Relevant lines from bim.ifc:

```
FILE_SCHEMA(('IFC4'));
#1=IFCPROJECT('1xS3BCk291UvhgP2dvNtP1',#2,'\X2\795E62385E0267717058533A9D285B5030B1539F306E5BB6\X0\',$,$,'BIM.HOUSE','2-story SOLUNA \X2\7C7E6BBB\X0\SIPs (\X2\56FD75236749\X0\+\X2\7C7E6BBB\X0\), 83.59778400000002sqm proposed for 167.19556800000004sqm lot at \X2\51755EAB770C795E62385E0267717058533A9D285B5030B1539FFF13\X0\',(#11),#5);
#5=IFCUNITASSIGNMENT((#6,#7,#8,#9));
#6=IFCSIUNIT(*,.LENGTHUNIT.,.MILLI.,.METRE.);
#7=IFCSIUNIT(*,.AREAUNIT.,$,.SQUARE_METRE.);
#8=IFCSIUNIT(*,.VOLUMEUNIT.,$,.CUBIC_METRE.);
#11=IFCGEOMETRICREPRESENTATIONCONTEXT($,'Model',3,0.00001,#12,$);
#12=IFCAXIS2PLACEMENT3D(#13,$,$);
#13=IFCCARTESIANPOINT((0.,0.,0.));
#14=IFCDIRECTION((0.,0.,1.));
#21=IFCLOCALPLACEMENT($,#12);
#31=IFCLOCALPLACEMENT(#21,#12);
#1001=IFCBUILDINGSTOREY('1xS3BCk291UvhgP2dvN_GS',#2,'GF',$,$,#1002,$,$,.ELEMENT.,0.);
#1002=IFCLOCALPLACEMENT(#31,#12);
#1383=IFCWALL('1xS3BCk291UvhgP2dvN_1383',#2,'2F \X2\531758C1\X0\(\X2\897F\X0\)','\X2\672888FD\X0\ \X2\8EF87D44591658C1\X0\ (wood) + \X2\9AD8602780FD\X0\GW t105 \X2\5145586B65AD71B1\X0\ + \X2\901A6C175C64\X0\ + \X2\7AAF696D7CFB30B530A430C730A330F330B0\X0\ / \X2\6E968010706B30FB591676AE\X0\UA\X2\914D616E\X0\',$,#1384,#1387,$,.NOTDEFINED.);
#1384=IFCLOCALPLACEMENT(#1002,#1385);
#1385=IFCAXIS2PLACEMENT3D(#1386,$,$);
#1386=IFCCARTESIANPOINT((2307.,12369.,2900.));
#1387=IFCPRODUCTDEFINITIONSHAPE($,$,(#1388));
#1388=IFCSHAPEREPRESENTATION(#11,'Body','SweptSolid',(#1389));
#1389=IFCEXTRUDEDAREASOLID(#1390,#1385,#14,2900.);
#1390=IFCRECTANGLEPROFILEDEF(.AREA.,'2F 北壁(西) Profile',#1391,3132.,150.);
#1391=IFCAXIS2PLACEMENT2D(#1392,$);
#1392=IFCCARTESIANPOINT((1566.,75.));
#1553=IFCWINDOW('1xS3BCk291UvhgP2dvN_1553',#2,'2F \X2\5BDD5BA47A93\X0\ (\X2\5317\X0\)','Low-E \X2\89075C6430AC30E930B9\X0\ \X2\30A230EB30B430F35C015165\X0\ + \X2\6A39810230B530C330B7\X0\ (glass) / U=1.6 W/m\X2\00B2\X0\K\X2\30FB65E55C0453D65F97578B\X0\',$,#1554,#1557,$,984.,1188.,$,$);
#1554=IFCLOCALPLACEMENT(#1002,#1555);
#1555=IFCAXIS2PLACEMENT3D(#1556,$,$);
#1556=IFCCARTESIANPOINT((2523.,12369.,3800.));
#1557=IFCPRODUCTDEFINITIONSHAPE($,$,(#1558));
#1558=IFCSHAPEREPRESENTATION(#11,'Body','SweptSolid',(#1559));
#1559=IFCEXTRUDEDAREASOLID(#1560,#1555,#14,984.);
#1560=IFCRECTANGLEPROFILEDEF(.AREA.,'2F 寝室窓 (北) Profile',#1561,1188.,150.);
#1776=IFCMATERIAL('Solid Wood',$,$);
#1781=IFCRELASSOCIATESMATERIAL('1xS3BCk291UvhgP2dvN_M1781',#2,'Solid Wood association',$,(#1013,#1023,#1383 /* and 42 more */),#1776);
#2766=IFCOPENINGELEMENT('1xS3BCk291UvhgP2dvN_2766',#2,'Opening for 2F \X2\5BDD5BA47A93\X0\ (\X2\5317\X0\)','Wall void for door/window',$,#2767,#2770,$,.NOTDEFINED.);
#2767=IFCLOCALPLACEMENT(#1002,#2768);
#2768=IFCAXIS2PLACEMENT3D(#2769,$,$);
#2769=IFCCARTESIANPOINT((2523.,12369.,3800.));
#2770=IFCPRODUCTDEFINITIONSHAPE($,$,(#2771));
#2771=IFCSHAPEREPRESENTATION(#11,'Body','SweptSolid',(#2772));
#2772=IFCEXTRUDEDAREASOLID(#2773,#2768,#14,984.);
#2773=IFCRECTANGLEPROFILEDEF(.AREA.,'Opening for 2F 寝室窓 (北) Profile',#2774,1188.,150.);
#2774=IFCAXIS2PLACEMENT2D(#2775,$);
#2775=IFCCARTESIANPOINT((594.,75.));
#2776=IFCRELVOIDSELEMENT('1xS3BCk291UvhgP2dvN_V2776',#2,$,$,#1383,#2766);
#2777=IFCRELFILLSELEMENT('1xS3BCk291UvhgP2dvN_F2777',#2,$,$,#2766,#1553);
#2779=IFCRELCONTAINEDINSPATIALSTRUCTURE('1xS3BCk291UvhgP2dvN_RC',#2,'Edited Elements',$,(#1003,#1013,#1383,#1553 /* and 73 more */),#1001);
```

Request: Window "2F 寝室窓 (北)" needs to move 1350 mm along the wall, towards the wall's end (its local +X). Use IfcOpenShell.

```python
import ifcopenshell
import ifcopenshell.api.geometry
import ifcopenshell.util.placement
import ifcopenshell.util.unit

model = ifcopenshell.open("bim.ifc")
unit_scale = ifcopenshell.util.unit.calculate_unit_scale(model)

window = model.by_guid("1xS3BCk291UvhgP2dvN_1553")
opening = window.FillsVoids[0].RelatingOpeningElement
wall = opening.VoidsElements[0].RelatingBuildingElement

wall_matrix = ifcopenshell.util.placement.get_local_placement(wall.ObjectPlacement)
shift = wall_matrix[:3, 0] * 1.35 / unit_scale
before = ifcopenshell.util.placement.get_local_placement(window.ObjectPlacement)[:3, 3].copy()

# The window is not placed relative to its opening, so move both.
for product in (opening, window):
    matrix = ifcopenshell.util.placement.get_local_placement(product.ObjectPlacement)
    matrix[:3, 3] += shift
    ifcopenshell.api.geometry.edit_object_placement(model, product=product, matrix=matrix, is_si=False)

after = ifcopenshell.util.placement.get_local_placement(window.ObjectPlacement)[:3, 3]
print("window moved by", (after - before).round(3) + 0.0)

model.write("bim_updated.ifc")
```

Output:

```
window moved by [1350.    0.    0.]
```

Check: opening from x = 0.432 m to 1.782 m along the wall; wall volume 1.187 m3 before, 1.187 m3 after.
